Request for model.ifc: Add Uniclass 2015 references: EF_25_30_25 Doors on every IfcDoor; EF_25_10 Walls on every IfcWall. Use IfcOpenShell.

First a look at what the model holds.

```python
import ifcopenshell

model = ifcopenshell.open("model.ifc")
print(model.schema)
print("classifications:", [c.Name for c in model.by_type("IfcClassification")])
for ifc_class in ("IfcDoor", "IfcRoof", "IfcStair", "IfcWall", "IfcWindow"):
    print(ifc_class, len(model.by_type(ifc_class)))
```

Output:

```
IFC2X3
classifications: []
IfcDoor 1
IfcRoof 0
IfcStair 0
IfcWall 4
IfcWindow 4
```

```python
import ifcopenshell
import ifcopenshell.api.classification

model = ifcopenshell.open("model.ifc")

# IFC2X3 requires Source and Edition and has no link from the project to the system.
system = model.create_entity("IfcClassification", Source="NBS", Edition="2015", Name="Uniclass 2015")

codes = {
    "IfcDoor": ("EF_25_30_25", "Doors"),
    "IfcWall": ("EF_25_10", "Walls"),
}
for ifc_class, (code, name) in codes.items():
    products = model.by_type(ifc_class)
    ifcopenshell.api.classification.add_reference(
        model, products=products, classification=system, identification=code, name=name
    )
    print(code, len(products))

model.write("model_updated.ifc")
```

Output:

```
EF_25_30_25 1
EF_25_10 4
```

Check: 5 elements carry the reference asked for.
